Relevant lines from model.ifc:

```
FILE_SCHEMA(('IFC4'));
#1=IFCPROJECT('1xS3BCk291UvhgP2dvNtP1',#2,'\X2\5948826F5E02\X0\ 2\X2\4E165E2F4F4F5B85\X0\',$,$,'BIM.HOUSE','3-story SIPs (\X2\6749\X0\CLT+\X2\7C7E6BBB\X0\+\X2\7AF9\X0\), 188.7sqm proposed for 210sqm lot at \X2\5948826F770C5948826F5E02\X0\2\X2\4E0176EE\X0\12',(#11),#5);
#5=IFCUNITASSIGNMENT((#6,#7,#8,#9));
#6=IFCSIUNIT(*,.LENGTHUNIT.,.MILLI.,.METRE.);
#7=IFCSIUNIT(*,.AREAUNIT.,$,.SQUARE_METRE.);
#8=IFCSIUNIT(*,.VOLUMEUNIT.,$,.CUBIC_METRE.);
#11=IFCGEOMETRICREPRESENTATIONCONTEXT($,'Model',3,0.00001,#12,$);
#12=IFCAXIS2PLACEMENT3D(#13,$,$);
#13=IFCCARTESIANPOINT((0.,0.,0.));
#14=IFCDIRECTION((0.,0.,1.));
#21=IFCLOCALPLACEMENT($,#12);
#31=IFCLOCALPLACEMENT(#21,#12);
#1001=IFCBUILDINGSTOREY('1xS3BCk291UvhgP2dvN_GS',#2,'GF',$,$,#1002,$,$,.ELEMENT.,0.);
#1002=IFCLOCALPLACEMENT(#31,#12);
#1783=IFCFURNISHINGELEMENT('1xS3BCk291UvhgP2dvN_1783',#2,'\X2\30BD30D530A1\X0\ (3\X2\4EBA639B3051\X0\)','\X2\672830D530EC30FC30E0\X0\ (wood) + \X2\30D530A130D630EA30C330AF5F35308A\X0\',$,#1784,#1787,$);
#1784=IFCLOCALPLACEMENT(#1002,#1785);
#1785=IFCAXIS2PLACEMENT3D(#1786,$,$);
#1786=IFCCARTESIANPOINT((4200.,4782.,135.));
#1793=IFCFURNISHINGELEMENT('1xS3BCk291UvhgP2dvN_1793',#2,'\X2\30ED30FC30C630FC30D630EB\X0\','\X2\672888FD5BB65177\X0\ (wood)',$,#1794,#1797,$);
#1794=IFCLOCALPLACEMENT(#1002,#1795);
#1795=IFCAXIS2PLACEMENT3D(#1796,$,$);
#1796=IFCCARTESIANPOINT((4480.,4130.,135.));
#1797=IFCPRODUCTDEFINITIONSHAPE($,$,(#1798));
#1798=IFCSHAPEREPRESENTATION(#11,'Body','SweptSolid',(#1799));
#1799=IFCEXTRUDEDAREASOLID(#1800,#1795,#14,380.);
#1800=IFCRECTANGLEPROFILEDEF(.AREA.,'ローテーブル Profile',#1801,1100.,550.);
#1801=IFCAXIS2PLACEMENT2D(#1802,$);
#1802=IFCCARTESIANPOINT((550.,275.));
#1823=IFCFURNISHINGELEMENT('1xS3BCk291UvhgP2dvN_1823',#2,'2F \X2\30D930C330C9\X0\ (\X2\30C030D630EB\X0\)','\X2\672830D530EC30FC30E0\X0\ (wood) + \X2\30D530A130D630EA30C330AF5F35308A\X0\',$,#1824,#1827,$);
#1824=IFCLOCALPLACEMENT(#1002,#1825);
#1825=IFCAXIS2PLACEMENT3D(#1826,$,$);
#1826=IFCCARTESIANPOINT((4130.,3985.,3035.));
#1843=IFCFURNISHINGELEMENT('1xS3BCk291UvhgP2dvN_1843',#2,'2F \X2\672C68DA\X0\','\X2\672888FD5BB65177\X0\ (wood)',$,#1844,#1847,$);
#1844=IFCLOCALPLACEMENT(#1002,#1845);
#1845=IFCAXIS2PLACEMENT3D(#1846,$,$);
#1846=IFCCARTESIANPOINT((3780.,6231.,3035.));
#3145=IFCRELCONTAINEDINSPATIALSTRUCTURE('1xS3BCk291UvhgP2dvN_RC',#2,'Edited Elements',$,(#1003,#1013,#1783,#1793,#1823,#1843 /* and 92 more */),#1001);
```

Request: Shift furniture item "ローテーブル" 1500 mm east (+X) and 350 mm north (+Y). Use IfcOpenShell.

```python
import ifcopenshell
import ifcopenshell.api.geometry
import ifcopenshell.util.placement

model = ifcopenshell.open("model.ifc")

item = model.by_guid("1xS3BCk291UvhgP2dvN_1793")
matrix = ifcopenshell.util.placement.get_local_placement(item.ObjectPlacement)
matrix[0, 3] += 1500.0
matrix[1, 3] += 350.0
ifcopenshell.api.geometry.edit_object_placement(model, product=item, matrix=matrix, is_si=False)

print(ifcopenshell.util.placement.get_local_placement(item.ObjectPlacement).round(3) + 0.0)

model.write("model_rev.ifc")
```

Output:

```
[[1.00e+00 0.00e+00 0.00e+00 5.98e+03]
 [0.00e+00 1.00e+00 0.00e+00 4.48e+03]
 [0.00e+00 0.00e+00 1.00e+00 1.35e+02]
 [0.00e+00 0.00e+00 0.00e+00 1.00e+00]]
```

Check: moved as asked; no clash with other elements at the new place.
